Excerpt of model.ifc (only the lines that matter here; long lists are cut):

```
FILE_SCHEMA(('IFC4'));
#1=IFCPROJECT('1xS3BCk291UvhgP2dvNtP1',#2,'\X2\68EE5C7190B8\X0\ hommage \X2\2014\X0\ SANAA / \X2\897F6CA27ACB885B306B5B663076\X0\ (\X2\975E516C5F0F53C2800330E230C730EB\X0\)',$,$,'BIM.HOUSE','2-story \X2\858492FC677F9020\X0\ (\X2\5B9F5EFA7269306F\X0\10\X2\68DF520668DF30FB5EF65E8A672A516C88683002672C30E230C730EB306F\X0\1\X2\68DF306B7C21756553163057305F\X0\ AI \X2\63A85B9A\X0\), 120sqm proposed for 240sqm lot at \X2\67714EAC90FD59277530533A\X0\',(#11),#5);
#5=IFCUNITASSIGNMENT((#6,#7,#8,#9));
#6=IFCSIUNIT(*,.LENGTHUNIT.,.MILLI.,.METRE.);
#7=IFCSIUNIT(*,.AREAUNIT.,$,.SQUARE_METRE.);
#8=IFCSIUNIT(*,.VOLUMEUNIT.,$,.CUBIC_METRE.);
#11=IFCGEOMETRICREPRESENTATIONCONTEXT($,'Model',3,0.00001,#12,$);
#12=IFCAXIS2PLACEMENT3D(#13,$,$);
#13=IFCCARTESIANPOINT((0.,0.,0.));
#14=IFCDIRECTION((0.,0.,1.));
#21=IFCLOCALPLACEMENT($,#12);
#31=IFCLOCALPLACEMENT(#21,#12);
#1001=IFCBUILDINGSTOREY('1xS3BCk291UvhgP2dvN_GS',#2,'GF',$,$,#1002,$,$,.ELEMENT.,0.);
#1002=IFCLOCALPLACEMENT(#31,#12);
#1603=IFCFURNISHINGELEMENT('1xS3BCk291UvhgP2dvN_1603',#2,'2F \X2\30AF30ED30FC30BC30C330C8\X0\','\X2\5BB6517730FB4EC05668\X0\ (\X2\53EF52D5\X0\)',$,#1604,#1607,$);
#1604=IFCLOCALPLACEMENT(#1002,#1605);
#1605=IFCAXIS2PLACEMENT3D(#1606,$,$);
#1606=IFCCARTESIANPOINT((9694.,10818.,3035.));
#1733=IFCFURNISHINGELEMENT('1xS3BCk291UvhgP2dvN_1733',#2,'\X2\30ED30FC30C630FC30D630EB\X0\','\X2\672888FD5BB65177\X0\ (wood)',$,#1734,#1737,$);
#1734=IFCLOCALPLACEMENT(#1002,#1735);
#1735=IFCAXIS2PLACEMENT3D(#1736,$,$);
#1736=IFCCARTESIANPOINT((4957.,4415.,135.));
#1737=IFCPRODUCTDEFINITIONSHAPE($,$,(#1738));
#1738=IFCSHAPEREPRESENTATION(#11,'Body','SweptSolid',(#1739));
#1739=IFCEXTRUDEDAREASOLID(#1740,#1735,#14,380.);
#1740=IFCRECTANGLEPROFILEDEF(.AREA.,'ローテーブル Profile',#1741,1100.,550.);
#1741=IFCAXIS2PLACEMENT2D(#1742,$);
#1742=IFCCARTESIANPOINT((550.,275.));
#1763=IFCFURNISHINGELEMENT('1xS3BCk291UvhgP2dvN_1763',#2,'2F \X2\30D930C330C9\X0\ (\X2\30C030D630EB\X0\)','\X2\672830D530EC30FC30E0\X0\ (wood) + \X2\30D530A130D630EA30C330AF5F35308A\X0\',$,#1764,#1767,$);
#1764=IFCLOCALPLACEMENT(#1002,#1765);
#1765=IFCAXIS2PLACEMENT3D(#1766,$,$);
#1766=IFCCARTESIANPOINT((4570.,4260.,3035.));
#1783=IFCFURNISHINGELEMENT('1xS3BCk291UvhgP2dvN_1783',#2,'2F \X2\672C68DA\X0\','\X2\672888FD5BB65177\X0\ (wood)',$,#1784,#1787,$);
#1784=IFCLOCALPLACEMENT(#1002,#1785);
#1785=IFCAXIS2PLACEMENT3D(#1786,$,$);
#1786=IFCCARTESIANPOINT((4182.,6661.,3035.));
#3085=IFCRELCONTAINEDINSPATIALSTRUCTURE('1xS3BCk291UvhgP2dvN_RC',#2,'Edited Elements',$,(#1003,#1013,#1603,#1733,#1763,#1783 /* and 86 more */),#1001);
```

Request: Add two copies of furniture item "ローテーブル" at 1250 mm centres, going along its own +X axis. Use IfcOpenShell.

```python
import ifcopenshell
import ifcopenshell.api.geometry
import ifcopenshell.api.root
import ifcopenshell.util.element
import ifcopenshell.util.placement
import ifcopenshell.util.unit

model = ifcopenshell.open("model.ifc")
unit_scale = ifcopenshell.util.unit.calculate_unit_scale(model)


def reuse_history(source, copy):
    """copy_class also copies each property set's owner history, people and application; keep the originals."""
    for rel in copy.IsDefinedBy:
        if rel.is_a("IfcRelDefinesByProperties") and (history := rel.RelatingPropertyDefinition.OwnerHistory):
            rel.RelatingPropertyDefinition.OwnerHistory = source.OwnerHistory
            ifcopenshell.util.element.remove_deep2(model, history)


source = model.by_guid("1xS3BCk291UvhgP2dvN_1733")
base = ifcopenshell.util.placement.get_local_placement(source.ObjectPlacement)
step = base[:3, 0] * 1.25 / unit_scale

for i in range(1, 3):
    copy = ifcopenshell.api.root.copy_class(model, product=source)
    copy.Representation = ifcopenshell.util.element.copy_deep(
        model, source.Representation, exclude=["IfcGeometricRepresentationContext", "IfcRepresentationMap"]
    )
    reuse_history(source, copy)
    matrix = base.copy()
    matrix[:3, 3] += i * step
    print("added at", matrix[:3, 3].round(3) + 0.0)
    ifcopenshell.api.geometry.edit_object_placement(model, product=copy, matrix=matrix, is_si=False)

model.write("model_v2.ifc")
```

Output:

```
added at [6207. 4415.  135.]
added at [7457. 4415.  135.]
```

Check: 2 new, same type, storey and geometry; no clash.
